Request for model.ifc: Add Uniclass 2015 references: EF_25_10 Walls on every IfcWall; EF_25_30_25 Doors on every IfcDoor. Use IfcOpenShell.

First a look at what the model holds.

```python
import ifcopenshell

model = ifcopenshell.open("model.ifc")
print(model.schema)
print("classifications:", [c.Name for c in model.by_type("IfcClassification")])
for ifc_class in ("IfcDoor", "IfcRoof", "IfcStair", "IfcWall", "IfcWindow"):
    print(ifc_class, len(model.by_type(ifc_class)))
```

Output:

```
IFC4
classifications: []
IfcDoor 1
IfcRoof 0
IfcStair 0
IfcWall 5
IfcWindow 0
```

```python
import ifcopenshell
import ifcopenshell.api.classification

model = ifcopenshell.open("model.ifc")

system = ifcopenshell.api.classification.add_classification(model, classification="Uniclass 2015")

codes = {
    "IfcWall": ("EF_25_10", "Walls"),
    "IfcDoor": ("EF_25_30_25", "Doors"),
}
for ifc_class, (code, name) in codes.items():
    products = model.by_type(ifc_class)
    ifcopenshell.api.classification.add_reference(
        model, products=products, classification=system, identification=code, name=name
    )
    print(code, len(products))

model.write("model_rev.ifc")
```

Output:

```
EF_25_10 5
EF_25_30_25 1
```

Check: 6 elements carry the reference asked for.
